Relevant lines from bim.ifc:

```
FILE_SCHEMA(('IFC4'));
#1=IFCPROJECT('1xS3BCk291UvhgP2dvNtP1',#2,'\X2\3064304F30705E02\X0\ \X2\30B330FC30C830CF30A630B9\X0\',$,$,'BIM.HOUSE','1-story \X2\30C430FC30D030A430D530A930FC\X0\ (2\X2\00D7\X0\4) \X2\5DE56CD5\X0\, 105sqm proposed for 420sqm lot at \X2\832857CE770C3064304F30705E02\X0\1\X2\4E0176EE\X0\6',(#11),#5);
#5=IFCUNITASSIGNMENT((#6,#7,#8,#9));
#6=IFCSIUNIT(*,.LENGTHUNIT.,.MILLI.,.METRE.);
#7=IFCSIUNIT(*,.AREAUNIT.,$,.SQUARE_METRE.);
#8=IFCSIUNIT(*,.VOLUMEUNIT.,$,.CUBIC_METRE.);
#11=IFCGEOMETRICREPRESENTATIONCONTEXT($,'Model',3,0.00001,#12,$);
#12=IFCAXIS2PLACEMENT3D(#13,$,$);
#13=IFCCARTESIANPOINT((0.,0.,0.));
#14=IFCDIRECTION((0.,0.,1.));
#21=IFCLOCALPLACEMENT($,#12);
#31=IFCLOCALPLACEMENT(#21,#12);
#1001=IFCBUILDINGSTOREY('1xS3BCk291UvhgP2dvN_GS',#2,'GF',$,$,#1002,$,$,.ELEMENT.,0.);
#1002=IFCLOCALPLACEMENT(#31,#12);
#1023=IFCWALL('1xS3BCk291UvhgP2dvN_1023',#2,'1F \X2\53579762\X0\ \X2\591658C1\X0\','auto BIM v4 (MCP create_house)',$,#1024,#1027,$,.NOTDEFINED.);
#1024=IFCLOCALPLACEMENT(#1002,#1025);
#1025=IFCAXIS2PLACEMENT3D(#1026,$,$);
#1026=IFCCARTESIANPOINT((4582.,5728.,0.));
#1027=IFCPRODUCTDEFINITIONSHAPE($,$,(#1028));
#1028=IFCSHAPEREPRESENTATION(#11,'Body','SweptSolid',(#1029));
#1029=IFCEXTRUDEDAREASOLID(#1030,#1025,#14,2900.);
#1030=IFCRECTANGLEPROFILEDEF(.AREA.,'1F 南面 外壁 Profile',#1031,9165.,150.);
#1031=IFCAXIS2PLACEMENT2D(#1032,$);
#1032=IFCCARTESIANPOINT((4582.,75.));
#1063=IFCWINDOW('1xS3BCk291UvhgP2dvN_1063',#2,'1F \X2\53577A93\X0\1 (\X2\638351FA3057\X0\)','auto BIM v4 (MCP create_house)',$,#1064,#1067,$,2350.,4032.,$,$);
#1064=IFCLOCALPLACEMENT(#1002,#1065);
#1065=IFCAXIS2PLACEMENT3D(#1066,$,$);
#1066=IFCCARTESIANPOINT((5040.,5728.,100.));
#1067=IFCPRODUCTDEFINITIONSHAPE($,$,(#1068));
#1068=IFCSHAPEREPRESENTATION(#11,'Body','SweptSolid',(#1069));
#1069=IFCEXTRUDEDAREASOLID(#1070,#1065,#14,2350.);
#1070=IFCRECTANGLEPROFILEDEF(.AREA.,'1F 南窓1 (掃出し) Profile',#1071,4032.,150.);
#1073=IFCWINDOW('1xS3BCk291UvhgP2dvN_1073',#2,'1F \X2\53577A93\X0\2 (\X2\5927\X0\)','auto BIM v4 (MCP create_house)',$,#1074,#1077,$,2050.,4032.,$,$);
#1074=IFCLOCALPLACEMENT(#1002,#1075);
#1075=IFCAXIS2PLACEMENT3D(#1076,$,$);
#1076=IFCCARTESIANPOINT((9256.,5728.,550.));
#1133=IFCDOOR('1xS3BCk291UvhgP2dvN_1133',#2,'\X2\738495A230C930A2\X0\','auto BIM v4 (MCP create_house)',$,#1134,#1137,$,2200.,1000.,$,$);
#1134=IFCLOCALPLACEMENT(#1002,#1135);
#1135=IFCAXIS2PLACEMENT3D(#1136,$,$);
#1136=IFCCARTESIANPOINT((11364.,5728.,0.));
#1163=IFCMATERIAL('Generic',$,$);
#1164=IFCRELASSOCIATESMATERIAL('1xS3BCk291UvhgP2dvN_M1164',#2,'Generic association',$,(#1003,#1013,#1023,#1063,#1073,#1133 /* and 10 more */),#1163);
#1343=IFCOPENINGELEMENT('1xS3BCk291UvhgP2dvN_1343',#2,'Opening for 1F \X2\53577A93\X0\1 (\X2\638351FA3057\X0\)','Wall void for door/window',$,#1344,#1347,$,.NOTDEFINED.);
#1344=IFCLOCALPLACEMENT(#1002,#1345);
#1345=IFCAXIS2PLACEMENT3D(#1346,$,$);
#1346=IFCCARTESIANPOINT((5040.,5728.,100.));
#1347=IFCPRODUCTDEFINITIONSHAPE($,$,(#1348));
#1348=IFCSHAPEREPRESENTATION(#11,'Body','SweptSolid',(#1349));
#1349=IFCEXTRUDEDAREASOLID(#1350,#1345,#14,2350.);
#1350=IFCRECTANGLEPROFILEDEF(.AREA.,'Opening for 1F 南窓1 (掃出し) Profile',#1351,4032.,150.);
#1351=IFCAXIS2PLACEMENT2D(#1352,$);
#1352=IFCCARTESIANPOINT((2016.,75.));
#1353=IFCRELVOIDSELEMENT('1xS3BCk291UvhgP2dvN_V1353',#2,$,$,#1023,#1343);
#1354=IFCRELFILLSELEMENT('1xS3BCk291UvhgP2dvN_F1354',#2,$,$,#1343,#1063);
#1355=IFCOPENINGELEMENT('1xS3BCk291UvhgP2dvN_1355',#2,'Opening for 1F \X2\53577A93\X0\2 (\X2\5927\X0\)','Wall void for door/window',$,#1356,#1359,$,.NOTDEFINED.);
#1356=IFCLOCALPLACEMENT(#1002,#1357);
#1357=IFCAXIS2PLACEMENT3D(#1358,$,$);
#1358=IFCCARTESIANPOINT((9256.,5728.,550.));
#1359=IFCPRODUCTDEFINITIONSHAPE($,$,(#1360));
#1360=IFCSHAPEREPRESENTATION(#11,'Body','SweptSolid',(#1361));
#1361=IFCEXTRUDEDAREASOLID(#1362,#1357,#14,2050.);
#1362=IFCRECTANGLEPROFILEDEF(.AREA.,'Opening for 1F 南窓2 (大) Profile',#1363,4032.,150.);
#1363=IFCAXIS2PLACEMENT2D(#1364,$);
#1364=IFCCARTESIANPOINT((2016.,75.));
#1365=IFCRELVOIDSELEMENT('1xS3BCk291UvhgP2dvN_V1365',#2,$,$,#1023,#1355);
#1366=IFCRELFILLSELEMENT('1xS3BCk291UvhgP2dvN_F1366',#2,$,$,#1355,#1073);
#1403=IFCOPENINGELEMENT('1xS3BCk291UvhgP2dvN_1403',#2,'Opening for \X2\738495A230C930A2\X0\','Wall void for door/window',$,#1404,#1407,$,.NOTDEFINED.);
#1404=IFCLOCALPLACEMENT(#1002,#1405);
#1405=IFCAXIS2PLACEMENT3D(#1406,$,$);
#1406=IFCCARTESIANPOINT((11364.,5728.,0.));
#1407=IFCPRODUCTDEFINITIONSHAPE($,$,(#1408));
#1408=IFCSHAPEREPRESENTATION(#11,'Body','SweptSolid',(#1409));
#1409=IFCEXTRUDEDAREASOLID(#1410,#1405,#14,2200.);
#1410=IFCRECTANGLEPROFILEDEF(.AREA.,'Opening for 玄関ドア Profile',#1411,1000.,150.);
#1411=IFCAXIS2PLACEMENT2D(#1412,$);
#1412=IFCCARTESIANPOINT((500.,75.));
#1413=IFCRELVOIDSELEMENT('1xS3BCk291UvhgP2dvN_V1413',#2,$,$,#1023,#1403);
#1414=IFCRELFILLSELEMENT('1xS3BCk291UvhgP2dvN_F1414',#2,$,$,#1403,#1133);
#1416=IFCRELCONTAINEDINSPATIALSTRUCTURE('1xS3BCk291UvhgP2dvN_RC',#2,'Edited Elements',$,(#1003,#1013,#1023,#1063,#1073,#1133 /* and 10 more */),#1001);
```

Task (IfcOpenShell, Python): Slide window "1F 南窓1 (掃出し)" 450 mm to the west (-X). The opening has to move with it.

```python
import ifcopenshell
import ifcopenshell.api.geometry
import ifcopenshell.util.placement
import ifcopenshell.util.unit

model = ifcopenshell.open("bim.ifc")
unit_scale = ifcopenshell.util.unit.calculate_unit_scale(model)

window = model.by_guid("1xS3BCk291UvhgP2dvN_1063")
opening = window.FillsVoids[0].RelatingOpeningElement
wall = opening.VoidsElements[0].RelatingBuildingElement

wall_matrix = ifcopenshell.util.placement.get_local_placement(wall.ObjectPlacement)
shift = wall_matrix[:3, 0] * -0.45 / unit_scale
before = ifcopenshell.util.placement.get_local_placement(window.ObjectPlacement)[:3, 3].copy()

# The window is not placed relative to its opening, so move both.
for product in (opening, window):
    matrix = ifcopenshell.util.placement.get_local_placement(product.ObjectPlacement)
    matrix[:3, 3] += shift
    ifcopenshell.api.geometry.edit_object_placement(model, product=product, matrix=matrix, is_si=False)

after = ifcopenshell.util.placement.get_local_placement(window.ObjectPlacement)[:3, 3]
print("window moved by", (after - before).round(3) + 0.0)

model.write("bim_v2.ifc")
```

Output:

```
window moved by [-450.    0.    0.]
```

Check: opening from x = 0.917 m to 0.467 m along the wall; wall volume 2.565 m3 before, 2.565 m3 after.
